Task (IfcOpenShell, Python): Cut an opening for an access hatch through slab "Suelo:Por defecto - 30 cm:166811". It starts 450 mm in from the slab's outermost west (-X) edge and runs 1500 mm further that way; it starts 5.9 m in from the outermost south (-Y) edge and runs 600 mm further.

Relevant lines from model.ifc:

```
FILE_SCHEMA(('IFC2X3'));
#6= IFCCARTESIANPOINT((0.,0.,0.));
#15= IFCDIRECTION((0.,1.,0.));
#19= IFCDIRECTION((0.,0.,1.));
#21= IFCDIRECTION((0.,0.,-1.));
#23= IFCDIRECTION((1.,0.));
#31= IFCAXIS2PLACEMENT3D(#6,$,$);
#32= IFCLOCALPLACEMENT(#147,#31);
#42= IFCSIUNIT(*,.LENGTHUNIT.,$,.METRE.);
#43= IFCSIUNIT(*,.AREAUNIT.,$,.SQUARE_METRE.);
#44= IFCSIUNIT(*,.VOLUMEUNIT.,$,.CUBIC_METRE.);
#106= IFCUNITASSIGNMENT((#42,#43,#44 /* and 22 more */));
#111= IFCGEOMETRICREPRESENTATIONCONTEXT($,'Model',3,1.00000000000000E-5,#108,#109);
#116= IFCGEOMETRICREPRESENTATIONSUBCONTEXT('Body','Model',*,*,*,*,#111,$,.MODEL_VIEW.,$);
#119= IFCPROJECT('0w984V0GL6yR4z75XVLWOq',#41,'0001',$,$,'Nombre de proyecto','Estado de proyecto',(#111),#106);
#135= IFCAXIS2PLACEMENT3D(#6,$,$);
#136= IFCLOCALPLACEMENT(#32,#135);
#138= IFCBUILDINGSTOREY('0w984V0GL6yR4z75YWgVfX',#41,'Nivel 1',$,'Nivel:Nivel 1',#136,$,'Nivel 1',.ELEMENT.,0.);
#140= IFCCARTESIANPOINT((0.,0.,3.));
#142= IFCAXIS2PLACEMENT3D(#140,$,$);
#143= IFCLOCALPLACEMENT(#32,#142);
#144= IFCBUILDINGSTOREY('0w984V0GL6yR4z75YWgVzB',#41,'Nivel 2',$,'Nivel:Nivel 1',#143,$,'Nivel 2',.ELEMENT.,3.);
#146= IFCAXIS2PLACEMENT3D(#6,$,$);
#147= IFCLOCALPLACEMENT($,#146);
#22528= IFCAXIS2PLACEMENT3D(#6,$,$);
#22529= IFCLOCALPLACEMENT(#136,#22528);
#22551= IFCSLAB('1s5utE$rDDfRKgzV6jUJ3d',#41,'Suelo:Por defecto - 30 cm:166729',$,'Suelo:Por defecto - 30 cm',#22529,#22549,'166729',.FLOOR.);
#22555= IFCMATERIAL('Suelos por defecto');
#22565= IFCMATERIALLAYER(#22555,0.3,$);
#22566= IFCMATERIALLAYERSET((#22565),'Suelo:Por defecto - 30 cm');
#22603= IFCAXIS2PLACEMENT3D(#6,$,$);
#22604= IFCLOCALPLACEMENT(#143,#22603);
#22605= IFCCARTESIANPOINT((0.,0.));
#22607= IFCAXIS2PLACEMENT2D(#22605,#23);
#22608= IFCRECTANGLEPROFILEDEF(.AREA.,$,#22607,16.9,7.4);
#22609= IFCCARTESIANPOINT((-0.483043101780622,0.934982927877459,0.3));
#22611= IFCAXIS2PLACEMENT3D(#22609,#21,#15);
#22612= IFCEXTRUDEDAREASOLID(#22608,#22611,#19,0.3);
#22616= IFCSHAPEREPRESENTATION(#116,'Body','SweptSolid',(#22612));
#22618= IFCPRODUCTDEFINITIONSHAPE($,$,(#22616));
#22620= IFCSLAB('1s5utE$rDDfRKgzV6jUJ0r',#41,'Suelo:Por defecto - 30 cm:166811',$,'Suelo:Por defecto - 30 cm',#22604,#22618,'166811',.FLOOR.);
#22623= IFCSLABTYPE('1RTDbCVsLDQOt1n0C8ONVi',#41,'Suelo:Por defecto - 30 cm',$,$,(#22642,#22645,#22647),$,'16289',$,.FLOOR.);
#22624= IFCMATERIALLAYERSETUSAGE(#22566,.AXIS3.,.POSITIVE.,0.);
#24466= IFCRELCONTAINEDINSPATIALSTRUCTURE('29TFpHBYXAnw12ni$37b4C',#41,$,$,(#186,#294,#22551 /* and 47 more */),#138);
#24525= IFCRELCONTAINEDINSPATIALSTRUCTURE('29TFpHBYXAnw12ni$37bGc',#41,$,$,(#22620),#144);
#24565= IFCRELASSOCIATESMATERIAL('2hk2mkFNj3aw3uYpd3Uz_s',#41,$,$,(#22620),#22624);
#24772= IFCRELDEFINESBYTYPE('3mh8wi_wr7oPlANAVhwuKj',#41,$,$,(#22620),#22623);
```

```python
import numpy as np
import ifcopenshell
import ifcopenshell.api.feature
import ifcopenshell.api.geometry
import ifcopenshell.api.root
import ifcopenshell.geom
import ifcopenshell.util.placement
import ifcopenshell.util.representation
import ifcopenshell.util.shape
import ifcopenshell.util.unit

model = ifcopenshell.open("model.ifc")
unit_scale = ifcopenshell.util.unit.calculate_unit_scale(model)
settings = ifcopenshell.geom.settings()


def volume(element):
    """Net volume in cubic metres, openings subtracted."""
    shape = ifcopenshell.geom.create_shape(settings, element)
    return ifcopenshell.util.shape.get_volume(shape.geometry)


slab = model.by_id(22620)
before = volume(slab)

# Extent in the slab's own axes, in metres. The edges named are its -X and -Y sides.
slab_shape = ifcopenshell.geom.create_shape(settings, slab)
vertices = ifcopenshell.util.shape.get_vertices(slab_shape.geometry)
x_min, y_min, bottom = vertices.min(axis=0)
top = vertices[:, 2].max()

opening = ifcopenshell.api.root.create_entity(model, ifc_class="IfcOpeningElement", name="Access hatch opening")
context = ifcopenshell.util.representation.get_context(model, "Model", "Body", "MODEL_VIEW")
width, depth = 1.5, 0.6
outline = [(0.0, 0.0), (width, 0.0), (width, depth), (0.0, depth), (0.0, 0.0)]
# Overshoot both faces by 50 mm so the cut is clean.
shape = ifcopenshell.api.geometry.add_slab_representation(
    model, context=context, depth=top - bottom + 0.1, polyline=outline
)
ifcopenshell.api.geometry.assign_representation(model, product=opening, representation=shape)

matrix = ifcopenshell.util.placement.get_local_placement(slab.ObjectPlacement)
matrix[:, 3] = matrix @ np.append(np.array([x_min + 0.45, y_min + 5.9, bottom - 0.05]) / unit_scale, 1.0)
ifcopenshell.api.geometry.edit_object_placement(model, product=opening, matrix=matrix, is_si=False)
ifcopenshell.api.feature.add_feature(model, feature=opening, element=slab)

after = volume(slab)

print(f"slab volume {before:.3f} -> {after:.3f} m3")

model.write("model-out.ifc")
```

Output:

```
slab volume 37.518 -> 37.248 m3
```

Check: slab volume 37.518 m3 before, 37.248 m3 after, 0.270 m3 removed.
